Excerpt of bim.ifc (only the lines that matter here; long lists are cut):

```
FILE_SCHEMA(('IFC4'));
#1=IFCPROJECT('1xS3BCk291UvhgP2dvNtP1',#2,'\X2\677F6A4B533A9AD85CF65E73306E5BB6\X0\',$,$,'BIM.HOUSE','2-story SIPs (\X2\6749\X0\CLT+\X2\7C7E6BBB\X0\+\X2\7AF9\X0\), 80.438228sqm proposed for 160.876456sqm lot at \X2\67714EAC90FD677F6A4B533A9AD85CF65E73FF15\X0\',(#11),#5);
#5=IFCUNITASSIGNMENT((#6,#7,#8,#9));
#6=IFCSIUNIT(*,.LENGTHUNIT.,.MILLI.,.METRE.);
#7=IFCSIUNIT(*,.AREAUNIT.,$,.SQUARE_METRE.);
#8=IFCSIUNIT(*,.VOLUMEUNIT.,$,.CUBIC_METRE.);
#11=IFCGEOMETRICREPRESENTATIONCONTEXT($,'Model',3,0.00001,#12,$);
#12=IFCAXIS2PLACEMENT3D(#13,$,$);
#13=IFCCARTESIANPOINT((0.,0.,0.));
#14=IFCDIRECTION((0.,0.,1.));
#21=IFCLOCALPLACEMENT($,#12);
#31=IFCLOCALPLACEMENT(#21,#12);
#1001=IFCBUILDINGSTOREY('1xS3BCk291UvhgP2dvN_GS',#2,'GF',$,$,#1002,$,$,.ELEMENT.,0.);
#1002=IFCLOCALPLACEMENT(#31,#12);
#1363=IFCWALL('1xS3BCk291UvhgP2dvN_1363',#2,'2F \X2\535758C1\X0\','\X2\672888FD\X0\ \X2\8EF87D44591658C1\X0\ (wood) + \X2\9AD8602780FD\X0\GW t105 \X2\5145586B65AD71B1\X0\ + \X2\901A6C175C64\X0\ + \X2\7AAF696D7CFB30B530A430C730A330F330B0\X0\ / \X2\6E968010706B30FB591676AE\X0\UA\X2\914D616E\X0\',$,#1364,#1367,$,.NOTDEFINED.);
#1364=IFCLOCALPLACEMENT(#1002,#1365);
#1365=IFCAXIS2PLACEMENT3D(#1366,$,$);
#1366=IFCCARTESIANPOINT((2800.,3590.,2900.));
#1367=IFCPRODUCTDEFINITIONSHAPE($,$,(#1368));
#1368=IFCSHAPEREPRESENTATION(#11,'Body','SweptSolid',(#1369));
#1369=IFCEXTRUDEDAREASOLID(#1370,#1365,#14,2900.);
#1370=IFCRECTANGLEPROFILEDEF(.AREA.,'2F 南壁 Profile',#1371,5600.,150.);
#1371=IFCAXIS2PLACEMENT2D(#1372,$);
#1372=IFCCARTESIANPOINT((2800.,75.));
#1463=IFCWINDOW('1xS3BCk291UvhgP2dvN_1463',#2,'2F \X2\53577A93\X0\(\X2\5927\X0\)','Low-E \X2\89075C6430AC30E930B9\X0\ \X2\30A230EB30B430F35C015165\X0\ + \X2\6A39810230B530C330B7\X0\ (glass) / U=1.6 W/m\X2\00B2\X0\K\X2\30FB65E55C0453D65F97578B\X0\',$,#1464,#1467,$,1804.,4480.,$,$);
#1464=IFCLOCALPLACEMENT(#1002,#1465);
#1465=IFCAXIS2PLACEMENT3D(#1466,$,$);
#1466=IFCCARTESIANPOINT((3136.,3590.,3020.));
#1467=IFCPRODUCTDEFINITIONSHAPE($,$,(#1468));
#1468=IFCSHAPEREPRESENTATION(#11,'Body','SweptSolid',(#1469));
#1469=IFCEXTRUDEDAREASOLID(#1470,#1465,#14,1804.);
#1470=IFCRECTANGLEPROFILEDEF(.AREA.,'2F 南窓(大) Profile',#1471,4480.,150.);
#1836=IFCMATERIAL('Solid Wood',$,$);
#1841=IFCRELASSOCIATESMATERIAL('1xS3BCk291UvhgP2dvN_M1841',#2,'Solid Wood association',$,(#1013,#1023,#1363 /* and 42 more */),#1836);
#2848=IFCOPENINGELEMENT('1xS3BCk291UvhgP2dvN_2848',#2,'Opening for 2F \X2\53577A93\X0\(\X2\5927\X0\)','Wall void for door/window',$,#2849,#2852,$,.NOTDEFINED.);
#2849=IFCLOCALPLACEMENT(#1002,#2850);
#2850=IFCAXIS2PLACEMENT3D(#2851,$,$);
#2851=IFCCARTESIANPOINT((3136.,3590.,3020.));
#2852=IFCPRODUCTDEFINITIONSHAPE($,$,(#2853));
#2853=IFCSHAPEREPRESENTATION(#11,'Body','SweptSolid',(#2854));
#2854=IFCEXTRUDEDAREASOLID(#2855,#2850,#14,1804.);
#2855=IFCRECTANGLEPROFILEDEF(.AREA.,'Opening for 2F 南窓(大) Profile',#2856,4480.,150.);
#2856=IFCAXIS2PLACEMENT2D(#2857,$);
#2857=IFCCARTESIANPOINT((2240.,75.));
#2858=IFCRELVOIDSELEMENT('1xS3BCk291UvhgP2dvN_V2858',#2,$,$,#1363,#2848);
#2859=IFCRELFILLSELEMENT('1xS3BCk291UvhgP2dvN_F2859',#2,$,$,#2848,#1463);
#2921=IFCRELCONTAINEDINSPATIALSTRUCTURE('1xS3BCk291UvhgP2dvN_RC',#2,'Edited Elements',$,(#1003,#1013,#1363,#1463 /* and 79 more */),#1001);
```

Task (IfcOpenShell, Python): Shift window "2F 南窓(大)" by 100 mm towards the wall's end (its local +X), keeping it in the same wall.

```python
import ifcopenshell
import ifcopenshell.api.geometry
import ifcopenshell.util.placement
import ifcopenshell.util.unit

model = ifcopenshell.open("bim.ifc")
unit_scale = ifcopenshell.util.unit.calculate_unit_scale(model)

window = model.by_guid("1xS3BCk291UvhgP2dvN_1463")
opening = window.FillsVoids[0].RelatingOpeningElement
wall = opening.VoidsElements[0].RelatingBuildingElement

wall_matrix = ifcopenshell.util.placement.get_local_placement(wall.ObjectPlacement)
shift = wall_matrix[:3, 0] * 0.1 / unit_scale
before = ifcopenshell.util.placement.get_local_placement(window.ObjectPlacement)[:3, 3].copy()

# The window is not placed relative to its opening, so move both.
for product in (opening, window):
    matrix = ifcopenshell.util.placement.get_local_placement(product.ObjectPlacement)
    matrix[:3, 3] += shift
    ifcopenshell.api.geometry.edit_object_placement(model, product=product, matrix=matrix, is_si=False)

after = ifcopenshell.util.placement.get_local_placement(window.ObjectPlacement)[:3, 3]
print("window moved by", (after - before).round(3) + 0.0)

model.write("bim_rev.ifc")
```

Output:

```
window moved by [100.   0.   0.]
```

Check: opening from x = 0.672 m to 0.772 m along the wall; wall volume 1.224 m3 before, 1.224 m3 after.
